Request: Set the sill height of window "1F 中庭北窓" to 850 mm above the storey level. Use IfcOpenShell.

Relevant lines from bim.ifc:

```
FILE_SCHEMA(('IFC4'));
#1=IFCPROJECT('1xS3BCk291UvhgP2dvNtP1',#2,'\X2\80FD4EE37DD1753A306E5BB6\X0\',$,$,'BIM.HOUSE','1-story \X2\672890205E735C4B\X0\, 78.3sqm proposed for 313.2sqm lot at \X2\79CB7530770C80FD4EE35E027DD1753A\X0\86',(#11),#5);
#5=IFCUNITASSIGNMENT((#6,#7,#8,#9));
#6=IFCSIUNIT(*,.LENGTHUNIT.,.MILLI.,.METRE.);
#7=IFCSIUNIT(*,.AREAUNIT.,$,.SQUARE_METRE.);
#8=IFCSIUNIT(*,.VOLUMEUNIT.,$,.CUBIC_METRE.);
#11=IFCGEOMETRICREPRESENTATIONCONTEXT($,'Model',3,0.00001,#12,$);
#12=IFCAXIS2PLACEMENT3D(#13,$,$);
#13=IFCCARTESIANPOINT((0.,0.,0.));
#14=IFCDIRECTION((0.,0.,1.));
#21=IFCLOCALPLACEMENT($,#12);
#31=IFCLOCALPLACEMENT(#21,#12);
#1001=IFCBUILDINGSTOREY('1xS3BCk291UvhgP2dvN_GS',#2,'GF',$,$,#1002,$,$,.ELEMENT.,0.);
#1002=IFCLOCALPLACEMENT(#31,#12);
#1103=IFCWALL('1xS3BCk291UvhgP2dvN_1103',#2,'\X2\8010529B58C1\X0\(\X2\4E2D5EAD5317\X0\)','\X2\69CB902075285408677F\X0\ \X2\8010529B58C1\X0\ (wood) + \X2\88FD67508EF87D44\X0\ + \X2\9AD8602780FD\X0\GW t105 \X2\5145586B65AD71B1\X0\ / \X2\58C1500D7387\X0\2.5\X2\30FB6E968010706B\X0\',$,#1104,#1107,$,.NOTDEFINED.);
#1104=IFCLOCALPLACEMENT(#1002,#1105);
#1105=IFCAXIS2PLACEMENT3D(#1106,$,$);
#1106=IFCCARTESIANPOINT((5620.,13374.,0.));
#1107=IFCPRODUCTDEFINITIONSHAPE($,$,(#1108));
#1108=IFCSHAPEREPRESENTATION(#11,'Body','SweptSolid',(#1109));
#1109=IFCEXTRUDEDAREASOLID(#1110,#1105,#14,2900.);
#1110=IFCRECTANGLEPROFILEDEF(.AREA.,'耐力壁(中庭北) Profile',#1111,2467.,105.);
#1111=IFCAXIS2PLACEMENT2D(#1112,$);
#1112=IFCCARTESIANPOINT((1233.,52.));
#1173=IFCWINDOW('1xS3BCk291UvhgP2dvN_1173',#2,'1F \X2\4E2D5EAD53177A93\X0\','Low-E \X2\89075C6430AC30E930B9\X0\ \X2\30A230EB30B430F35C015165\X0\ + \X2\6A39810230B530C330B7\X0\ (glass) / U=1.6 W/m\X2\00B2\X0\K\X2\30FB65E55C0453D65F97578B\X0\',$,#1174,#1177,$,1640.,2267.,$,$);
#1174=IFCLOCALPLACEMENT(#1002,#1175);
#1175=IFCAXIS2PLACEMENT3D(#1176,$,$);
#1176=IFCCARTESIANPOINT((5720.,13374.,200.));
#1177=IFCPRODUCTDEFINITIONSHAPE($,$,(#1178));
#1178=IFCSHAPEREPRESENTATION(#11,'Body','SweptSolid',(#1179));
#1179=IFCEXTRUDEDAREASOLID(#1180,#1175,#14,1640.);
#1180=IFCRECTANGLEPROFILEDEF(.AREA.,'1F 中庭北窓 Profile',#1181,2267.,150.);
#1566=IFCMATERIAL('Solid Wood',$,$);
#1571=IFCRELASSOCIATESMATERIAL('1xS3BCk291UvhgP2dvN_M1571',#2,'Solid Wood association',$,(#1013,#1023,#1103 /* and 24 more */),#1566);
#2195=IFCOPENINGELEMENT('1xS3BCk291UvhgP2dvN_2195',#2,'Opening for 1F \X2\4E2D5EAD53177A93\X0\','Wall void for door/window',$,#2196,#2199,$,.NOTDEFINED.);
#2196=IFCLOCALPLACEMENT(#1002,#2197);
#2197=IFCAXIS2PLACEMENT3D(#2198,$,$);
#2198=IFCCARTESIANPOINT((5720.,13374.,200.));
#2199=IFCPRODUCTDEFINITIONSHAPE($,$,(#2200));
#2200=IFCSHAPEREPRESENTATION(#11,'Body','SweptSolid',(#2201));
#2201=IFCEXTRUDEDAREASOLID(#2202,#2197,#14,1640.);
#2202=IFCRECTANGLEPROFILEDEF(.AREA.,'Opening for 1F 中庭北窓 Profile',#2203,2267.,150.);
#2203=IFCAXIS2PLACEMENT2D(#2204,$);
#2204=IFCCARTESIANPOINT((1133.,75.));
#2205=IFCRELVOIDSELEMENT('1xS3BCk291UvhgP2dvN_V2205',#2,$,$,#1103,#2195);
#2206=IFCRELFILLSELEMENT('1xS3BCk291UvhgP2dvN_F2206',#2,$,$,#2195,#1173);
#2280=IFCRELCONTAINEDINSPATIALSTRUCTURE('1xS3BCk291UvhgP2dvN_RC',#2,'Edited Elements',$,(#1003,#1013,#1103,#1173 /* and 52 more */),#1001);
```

```python
import numpy as np
import ifcopenshell
import ifcopenshell.api.geometry
import ifcopenshell.geom
import ifcopenshell.util.element
import ifcopenshell.util.placement
import ifcopenshell.util.shape
import ifcopenshell.util.unit

model = ifcopenshell.open("bim.ifc")
unit_scale = ifcopenshell.util.unit.calculate_unit_scale(model)

window = model.by_guid("1xS3BCk291UvhgP2dvN_1173")
opening = window.FillsVoids[0].RelatingOpeningElement
storey = ifcopenshell.util.element.get_container(window, ifc_class="IfcBuildingStorey")
level = ifcopenshell.util.placement.get_local_placement(storey.ObjectPlacement)[2, 3]

# The opening's origin need not be at the sill, so measure its lowest point.
shape = ifcopenshell.geom.create_shape(ifcopenshell.geom.settings(), opening)
bottom = ifcopenshell.util.shape.get_shape_bottom_elevation(shape, shape.geometry) / unit_scale
dz = level + 0.85 / unit_scale - bottom

shift = np.array([0.0, 0.0, dz])
# The window is not placed relative to its opening, so move both.
for product in (opening, window):
    matrix = ifcopenshell.util.placement.get_local_placement(product.ObjectPlacement)
    matrix[:3, 3] += shift
    ifcopenshell.api.geometry.edit_object_placement(model, product=product, matrix=matrix, is_si=False)

print(f"moved by {dz * unit_scale:+.3f} m")

model.write("bim_edited.ifc")
```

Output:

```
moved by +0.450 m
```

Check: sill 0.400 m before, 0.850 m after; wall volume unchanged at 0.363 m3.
